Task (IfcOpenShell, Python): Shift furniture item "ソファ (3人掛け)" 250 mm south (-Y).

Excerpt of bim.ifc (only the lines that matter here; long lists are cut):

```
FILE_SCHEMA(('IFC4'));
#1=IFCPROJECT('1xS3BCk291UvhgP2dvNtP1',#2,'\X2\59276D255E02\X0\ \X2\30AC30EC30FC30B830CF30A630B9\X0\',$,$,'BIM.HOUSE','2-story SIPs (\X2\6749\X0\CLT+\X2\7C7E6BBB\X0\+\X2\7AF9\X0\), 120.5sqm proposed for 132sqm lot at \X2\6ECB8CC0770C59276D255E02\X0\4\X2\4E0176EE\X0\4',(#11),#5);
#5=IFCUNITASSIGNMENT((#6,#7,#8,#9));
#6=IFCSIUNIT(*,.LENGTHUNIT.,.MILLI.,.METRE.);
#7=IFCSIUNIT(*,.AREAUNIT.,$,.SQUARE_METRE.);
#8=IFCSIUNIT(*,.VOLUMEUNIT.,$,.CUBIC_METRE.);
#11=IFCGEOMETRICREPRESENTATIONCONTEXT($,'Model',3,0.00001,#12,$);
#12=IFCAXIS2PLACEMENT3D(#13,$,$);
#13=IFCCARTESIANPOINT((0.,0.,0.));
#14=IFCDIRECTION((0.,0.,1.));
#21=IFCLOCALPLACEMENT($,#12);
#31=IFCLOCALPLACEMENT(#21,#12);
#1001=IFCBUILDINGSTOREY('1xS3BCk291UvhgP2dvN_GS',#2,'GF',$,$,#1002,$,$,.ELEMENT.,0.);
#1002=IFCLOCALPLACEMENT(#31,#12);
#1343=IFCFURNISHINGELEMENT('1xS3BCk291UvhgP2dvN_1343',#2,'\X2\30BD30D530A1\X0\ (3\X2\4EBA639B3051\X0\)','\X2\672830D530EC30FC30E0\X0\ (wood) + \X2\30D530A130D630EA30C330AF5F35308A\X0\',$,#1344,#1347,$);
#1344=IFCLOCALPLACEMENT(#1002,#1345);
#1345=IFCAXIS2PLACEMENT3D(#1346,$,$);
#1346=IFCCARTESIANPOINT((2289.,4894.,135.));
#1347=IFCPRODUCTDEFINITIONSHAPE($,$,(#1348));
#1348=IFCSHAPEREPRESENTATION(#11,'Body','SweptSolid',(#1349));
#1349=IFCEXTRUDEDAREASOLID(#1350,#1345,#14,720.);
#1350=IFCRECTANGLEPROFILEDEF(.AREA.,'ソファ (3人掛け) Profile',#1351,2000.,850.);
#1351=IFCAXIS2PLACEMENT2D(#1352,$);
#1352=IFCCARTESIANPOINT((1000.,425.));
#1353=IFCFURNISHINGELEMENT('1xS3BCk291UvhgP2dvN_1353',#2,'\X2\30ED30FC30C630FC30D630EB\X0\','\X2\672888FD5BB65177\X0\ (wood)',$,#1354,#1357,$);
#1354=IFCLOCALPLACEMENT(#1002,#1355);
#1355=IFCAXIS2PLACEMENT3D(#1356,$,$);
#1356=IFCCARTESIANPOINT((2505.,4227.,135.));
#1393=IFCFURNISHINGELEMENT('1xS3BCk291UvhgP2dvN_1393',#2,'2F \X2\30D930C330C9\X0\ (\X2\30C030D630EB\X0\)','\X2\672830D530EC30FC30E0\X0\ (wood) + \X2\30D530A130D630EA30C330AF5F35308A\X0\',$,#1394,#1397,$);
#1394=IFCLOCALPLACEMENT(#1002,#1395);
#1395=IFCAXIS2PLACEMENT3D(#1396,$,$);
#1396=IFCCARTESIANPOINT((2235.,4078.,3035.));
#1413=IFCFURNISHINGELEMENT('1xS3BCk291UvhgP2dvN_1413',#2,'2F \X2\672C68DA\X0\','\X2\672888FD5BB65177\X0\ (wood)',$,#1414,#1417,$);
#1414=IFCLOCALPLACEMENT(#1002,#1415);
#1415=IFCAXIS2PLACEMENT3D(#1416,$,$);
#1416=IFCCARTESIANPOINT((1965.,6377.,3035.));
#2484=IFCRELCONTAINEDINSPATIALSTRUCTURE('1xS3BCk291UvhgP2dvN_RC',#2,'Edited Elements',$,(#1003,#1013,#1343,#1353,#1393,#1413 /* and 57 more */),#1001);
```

```python
import ifcopenshell
import ifcopenshell.api.geometry
import ifcopenshell.util.placement
import ifcopenshell.util.unit

model = ifcopenshell.open("bim.ifc")
unit_scale = ifcopenshell.util.unit.calculate_unit_scale(model)

item = model.by_guid("1xS3BCk291UvhgP2dvN_1343")
matrix = ifcopenshell.util.placement.get_local_placement(item.ObjectPlacement)
matrix[1, 3] -= 0.25 / unit_scale
ifcopenshell.api.geometry.edit_object_placement(model, product=item, matrix=matrix, is_si=False)

print(ifcopenshell.util.placement.get_local_placement(item.ObjectPlacement).round(3) + 0.0)

model.write("bim_rev.ifc")
```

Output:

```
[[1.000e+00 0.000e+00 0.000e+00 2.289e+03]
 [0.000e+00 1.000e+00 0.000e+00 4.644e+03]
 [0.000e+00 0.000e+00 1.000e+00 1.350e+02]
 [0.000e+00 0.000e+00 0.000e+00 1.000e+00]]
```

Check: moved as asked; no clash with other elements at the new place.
